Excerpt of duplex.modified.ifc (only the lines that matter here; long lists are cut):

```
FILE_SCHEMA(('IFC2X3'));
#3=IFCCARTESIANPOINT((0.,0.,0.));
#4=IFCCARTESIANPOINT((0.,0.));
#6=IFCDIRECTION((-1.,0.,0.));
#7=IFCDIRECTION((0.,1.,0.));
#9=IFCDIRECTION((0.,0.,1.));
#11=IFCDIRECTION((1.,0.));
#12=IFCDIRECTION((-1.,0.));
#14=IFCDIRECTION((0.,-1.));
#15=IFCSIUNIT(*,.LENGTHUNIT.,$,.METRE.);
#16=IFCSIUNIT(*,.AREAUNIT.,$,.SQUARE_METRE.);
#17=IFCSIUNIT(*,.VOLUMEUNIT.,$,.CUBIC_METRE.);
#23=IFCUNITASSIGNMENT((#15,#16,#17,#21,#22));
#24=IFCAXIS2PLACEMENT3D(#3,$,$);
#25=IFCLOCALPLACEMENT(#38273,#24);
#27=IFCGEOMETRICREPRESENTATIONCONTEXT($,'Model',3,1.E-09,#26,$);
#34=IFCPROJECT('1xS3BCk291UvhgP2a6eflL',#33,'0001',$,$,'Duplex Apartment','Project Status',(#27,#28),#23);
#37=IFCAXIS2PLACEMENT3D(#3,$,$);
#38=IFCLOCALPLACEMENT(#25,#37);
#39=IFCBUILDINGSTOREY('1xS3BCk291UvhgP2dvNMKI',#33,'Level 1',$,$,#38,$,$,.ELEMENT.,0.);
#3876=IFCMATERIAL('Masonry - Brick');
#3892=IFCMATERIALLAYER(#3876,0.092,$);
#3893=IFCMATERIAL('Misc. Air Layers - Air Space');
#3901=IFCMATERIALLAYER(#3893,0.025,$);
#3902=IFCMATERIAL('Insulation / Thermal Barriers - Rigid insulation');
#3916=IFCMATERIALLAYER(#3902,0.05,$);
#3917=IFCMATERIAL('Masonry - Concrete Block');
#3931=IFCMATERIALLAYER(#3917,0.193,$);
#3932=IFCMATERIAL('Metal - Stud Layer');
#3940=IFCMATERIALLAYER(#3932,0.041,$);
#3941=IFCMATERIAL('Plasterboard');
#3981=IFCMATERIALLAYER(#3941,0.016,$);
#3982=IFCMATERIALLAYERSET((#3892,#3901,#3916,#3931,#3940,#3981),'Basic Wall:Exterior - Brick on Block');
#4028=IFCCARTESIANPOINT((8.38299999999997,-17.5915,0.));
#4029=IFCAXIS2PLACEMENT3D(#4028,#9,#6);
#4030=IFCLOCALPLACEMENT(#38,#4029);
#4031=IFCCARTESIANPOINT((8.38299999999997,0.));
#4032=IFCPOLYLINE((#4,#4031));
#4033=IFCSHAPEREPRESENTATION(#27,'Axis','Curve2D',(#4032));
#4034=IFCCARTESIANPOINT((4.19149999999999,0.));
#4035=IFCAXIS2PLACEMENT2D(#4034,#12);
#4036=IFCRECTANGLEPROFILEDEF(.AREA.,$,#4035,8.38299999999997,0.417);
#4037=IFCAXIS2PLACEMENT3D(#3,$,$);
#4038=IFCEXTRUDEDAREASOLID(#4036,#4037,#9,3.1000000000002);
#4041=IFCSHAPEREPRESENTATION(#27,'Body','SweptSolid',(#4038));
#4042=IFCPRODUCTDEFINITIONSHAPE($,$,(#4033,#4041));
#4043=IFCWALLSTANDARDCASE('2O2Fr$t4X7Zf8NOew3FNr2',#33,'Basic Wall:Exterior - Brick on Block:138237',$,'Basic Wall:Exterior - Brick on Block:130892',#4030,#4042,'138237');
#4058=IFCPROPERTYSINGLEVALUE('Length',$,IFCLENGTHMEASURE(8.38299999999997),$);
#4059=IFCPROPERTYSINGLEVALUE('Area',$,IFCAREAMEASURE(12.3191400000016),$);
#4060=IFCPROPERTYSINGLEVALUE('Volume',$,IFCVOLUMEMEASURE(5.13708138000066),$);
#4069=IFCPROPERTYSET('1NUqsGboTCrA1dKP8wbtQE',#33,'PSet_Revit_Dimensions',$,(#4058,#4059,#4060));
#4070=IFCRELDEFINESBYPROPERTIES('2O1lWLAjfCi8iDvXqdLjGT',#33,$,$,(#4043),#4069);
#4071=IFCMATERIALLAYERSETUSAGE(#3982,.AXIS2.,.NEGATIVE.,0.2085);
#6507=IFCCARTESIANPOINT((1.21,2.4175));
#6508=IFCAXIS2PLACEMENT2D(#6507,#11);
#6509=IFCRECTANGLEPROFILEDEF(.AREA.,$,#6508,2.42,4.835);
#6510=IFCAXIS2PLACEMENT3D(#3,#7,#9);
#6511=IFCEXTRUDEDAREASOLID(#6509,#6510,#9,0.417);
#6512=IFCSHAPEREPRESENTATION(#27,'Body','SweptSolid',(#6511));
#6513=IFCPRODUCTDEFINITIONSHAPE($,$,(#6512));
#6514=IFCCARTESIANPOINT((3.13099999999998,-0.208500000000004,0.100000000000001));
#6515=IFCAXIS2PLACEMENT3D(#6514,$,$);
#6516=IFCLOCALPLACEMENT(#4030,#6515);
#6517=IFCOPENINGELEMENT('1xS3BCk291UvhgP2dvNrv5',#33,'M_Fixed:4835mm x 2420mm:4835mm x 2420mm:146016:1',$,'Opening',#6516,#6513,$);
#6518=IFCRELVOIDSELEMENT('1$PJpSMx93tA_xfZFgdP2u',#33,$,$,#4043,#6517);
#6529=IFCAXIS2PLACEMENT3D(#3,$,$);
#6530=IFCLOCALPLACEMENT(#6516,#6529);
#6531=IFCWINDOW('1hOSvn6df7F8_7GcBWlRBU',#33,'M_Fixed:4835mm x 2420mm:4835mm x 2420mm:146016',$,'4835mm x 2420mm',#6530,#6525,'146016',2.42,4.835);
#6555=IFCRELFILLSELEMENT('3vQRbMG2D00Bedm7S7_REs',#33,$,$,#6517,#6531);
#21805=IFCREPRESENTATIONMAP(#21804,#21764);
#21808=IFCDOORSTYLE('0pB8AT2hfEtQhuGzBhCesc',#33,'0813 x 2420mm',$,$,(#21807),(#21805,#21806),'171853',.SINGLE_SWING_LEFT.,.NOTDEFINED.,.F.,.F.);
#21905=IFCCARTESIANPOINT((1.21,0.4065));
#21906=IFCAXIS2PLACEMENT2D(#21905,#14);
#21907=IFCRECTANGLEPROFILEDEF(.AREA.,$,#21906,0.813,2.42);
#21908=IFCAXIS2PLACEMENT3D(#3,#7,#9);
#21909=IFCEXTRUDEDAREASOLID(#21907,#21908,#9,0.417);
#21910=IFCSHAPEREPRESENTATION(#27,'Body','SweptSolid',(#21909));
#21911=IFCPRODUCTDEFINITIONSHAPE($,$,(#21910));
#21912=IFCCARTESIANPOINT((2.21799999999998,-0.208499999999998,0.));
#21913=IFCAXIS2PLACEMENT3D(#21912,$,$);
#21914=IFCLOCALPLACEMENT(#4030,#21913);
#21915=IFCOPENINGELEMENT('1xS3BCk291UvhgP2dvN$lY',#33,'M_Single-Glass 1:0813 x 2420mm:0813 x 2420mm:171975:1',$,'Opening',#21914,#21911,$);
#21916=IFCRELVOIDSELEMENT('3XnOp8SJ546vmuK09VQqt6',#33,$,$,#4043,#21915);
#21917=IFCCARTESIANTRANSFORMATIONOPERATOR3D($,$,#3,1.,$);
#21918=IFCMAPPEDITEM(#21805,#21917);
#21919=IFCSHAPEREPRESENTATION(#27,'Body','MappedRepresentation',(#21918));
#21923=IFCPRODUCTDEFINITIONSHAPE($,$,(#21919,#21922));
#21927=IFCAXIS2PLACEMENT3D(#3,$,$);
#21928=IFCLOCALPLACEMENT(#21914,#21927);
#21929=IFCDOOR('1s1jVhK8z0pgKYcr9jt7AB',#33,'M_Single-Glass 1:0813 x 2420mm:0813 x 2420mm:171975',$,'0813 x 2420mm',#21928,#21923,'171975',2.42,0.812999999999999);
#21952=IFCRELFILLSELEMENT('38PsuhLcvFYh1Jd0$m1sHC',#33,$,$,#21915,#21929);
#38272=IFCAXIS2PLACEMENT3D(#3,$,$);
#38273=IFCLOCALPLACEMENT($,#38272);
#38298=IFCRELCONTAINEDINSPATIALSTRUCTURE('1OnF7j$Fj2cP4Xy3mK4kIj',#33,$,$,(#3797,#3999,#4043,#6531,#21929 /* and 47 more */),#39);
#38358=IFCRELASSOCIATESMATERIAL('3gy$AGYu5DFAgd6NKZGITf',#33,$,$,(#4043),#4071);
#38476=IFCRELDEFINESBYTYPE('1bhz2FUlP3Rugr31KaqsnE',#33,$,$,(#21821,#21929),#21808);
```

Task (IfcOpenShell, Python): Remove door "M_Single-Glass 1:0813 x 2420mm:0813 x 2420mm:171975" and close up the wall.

```python
import ifcopenshell
import ifcopenshell.api.feature
import ifcopenshell.api.pset
import ifcopenshell.api.root
import ifcopenshell.geom
import ifcopenshell.util.element
import ifcopenshell.util.shape
import ifcopenshell.util.unit

model = ifcopenshell.open("duplex.modified.ifc")
area_scale = ifcopenshell.util.unit.calculate_unit_scale(model, "AREAUNIT")
volume_scale = ifcopenshell.util.unit.calculate_unit_scale(model, "VOLUMEUNIT")
settings = ifcopenshell.geom.settings()


def volume(element):
    """Net volume in cubic metres, openings subtracted."""
    shape = ifcopenshell.geom.create_shape(settings, element)
    return ifcopenshell.util.shape.get_volume(shape.geometry)


door = model.by_guid("1s1jVhK8z0pgKYcr9jt7AB")
opening = door.FillsVoids[0].RelatingOpeningElement
wall = opening.VoidsElements[0].RelatingBuildingElement
before = volume(wall)

ifcopenshell.api.root.remove_product(model, product=door)
ifcopenshell.api.feature.remove_feature(model, feature=opening)

after = volume(wall)
thickness = 0.417  # wall thickness in metres

# Update the wall's stored quantities.
pset = model.by_id(ifcopenshell.util.element.get_pset(wall, "PSet_Revit_Dimensions", should_inherit=False)["id"])
ifcopenshell.api.pset.edit_pset(model, pset=pset, properties={
    "Area": model.create_entity("IfcAreaMeasure", after / thickness / area_scale),
    "Volume": model.create_entity("IfcVolumeMeasure", after / volume_scale),
})

print(f"wall volume {before:.3f} -> {after:.3f} m3")

model.write("duplex.modified_edited.ifc")
```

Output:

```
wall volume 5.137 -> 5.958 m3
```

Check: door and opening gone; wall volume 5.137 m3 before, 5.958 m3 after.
